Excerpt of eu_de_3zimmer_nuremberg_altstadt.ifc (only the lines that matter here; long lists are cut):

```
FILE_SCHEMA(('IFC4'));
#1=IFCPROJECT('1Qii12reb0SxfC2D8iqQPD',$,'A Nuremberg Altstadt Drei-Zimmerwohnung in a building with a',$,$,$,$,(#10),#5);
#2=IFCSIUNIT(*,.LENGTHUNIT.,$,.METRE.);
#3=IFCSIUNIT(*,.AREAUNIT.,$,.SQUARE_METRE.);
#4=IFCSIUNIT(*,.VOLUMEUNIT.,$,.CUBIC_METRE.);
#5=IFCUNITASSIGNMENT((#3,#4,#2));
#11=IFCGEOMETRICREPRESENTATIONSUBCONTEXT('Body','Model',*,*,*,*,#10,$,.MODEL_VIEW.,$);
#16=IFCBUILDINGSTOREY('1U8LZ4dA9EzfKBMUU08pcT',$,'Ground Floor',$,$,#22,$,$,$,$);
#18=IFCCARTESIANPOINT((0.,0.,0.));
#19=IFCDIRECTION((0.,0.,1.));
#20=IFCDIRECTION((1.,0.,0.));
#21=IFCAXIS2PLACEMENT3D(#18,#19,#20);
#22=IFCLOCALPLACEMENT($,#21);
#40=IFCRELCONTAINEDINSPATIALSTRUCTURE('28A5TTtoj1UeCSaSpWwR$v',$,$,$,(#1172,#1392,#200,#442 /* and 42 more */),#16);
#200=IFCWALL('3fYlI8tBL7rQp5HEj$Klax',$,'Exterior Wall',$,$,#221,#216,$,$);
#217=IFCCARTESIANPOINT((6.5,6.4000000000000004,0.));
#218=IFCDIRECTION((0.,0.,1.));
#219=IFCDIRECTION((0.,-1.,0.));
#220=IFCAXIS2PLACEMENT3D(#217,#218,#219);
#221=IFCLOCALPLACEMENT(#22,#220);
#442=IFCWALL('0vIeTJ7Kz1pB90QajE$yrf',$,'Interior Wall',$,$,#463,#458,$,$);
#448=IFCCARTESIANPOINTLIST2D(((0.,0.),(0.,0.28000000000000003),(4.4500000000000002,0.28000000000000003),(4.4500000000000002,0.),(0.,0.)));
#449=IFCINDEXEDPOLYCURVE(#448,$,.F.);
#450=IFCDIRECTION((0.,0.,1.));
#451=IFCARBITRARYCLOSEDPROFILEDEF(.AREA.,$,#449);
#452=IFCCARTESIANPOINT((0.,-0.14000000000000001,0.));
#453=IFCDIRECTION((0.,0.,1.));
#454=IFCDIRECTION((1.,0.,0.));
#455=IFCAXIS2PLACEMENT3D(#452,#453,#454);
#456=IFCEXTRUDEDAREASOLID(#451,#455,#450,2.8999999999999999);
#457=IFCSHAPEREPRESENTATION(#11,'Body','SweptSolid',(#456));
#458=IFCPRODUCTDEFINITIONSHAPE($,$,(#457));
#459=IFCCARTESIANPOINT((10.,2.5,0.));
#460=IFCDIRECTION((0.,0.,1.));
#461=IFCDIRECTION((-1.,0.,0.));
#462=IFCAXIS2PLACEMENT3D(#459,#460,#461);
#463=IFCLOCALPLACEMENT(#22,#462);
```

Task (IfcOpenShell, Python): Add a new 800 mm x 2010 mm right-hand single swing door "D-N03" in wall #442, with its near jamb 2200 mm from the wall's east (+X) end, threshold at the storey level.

```python
import numpy as np
import ifcopenshell
import ifcopenshell.api.feature
import ifcopenshell.api.geometry
import ifcopenshell.api.root
import ifcopenshell.api.spatial
import ifcopenshell.geom
import ifcopenshell.util.element
import ifcopenshell.util.placement
import ifcopenshell.util.representation
import ifcopenshell.util.shape
import ifcopenshell.util.unit

model = ifcopenshell.open("eu_de_3zimmer_nuremberg_altstadt.ifc")
unit_scale = ifcopenshell.util.unit.calculate_unit_scale(model)
settings = ifcopenshell.geom.settings()


def volume(element):
    """Net volume in cubic metres, openings subtracted."""
    shape = ifcopenshell.geom.create_shape(settings, element)
    return ifcopenshell.util.shape.get_volume(shape.geometry)


wall = model.by_guid("0vIeTJ7Kz1pB90QajE$yrf")
storey = ifcopenshell.util.element.get_container(wall, ifc_class="IfcBuildingStorey")
context = ifcopenshell.util.representation.get_context(model, "Model", "Body", "MODEL_VIEW")
before = volume(wall)

width, height, from_end, sill = 0.8, 2.01, 2.2, 0.0  # metres

# The wall runs along its own X axis, and the end named is its -X end.
wall_shape = ifcopenshell.geom.create_shape(settings, wall)
x, y, z = ifcopenshell.util.shape.get_vertices(wall_shape.geometry).T
start = x.min() + from_end
face, thickness = float(y.min()), float(y.max() - y.min())
wall_matrix = ifcopenshell.util.placement.get_local_placement(wall.ObjectPlacement)
level = ifcopenshell.util.placement.get_local_placement(storey.ObjectPlacement)[2, 3]


def in_wall(x, y):
    """Placement at x, y metres in the wall's axes, at sill height."""
    matrix = wall_matrix.copy()
    matrix[:, 3] = wall_matrix @ np.array([x / unit_scale, y / unit_scale, 0.0, 1.0])
    matrix[2, 3] = level + sill / unit_scale
    return matrix


# Opening: a box that overshoots both wall faces by 50 mm.
opening = ifcopenshell.api.root.create_entity(model, ifc_class="IfcOpeningElement", predefined_type="OPENING")
box = ifcopenshell.api.geometry.add_wall_representation(
    model, context=context, length=width, height=height, thickness=thickness + 0.1
)
ifcopenshell.api.geometry.assign_representation(model, product=opening, representation=box)
ifcopenshell.api.geometry.edit_object_placement(model, product=opening, matrix=in_wall(start, face - 0.05), is_si=False)
ifcopenshell.api.feature.add_feature(model, feature=opening, element=wall)

door = ifcopenshell.api.root.create_entity(model, ifc_class="IfcDoor", name="D-N03", predefined_type="DOOR")
door.OverallWidth, door.OverallHeight = width / unit_scale, height / unit_scale
door.OperationType = "SINGLE_SWING_RIGHT"
body = ifcopenshell.api.geometry.add_door_representation(
    model,
    context=context,
    overall_width=door.OverallWidth,
    overall_height=door.OverallHeight,
    operation_type="SINGLE_SWING_RIGHT",
    lining_properties={"LiningDepth": thickness / unit_scale, "ThresholdDepth": thickness / unit_scale},
)
ifcopenshell.api.geometry.assign_representation(model, product=door, representation=body)
ifcopenshell.api.spatial.assign_container(model, products=[door], relating_structure=storey)
ifcopenshell.api.feature.add_filling(model, opening=opening, element=door)

# The lining spans the wall, so the door starts at the wall face.
ifcopenshell.api.geometry.edit_object_placement(model, product=door, matrix=in_wall(start, face), is_si=False)

after = volume(wall)

print(f"wall volume {before:.3f} -> {after:.3f} m3")

model.write("eu_de_3zimmer_nuremberg_altstadt_updated.ifc")
```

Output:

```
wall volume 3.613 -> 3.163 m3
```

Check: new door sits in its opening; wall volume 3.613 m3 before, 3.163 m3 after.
